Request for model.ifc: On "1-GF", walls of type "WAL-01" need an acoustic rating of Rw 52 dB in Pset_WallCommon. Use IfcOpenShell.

First a look at what the model holds.

```python
import ifcopenshell
import ifcopenshell.util.element

model = ifcopenshell.open("model.ifc")
print(model.schema)
storey = next(s for s in model.by_type("IfcBuildingStorey") if s.Name == "1-GF")
walls = [e for e in ifcopenshell.util.element.get_decomposition(storey) if e.is_a("IfcWall")]
seen = {}
for e in walls:
    element_type = ifcopenshell.util.element.get_type(e)
    key = (element_type.Name if element_type != e and element_type else None, ifcopenshell.util.element.get_pset(e, "Pset_WallCommon", "AcousticRating"))
    seen[key] = seen.get(key, 0) + 1
for (name, value), count in sorted(seen.items(), key=str):
    print(count, "x", name, "|", value)
```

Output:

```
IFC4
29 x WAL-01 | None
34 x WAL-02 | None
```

```python
import ifcopenshell
import ifcopenshell.api.pset
import ifcopenshell.util.element

model = ifcopenshell.open("model.ifc")

storey = next(s for s in model.by_type("IfcBuildingStorey") if s.Name == "1-GF")
walls = [e for e in ifcopenshell.util.element.get_decomposition(storey) if e.is_a("IfcWall")]

count = 0
for e in walls:
    element_type = ifcopenshell.util.element.get_type(e)
    if element_type in (None, e) or element_type.Name != "WAL-01":
        continue
    # add_pset returns the element's existing set when there is one.
    pset = ifcopenshell.api.pset.add_pset(model, product=e, name="Pset_WallCommon")
    ifcopenshell.api.pset.edit_pset(model, pset=pset, properties={"AcousticRating": "Rw 52 dB"})
    count += 1

print(count, "walls updated")

model.write("model_updated.ifc")
```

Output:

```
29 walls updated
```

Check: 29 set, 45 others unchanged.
